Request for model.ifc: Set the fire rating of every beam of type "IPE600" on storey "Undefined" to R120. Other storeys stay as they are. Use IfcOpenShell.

First a look at what the model holds.

```python
import ifcopenshell
import ifcopenshell.util.element

model = ifcopenshell.open("model.ifc")
print(model.schema)
storey = next(s for s in model.by_type("IfcBuildingStorey") if s.Name == "Undefined")
beams = [e for e in ifcopenshell.util.element.get_decomposition(storey) if e.is_a("IfcBeam")]
seen = {}
for e in beams:
    element_type = ifcopenshell.util.element.get_type(e)
    key = (element_type.Name if element_type != e and element_type else None, ifcopenshell.util.element.get_pset(e, "Pset_BeamCommon", "FireRating"))
    seen[key] = seen.get(key, 0) + 1
for (name, value), count in sorted(seen.items(), key=str):
    print(count, "x", name, "|", value)
```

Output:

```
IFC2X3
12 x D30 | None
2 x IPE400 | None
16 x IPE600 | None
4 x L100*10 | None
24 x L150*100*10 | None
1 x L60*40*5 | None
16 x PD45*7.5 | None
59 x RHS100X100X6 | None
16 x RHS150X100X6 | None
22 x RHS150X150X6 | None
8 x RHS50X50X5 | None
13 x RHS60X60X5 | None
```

```python
import ifcopenshell
import ifcopenshell.api.pset
import ifcopenshell.util.element

model = ifcopenshell.open("model.ifc")

storey = next(s for s in model.by_type("IfcBuildingStorey") if s.Name == "Undefined")
beams = [e for e in ifcopenshell.util.element.get_decomposition(storey) if e.is_a("IfcBeam")]

count = 0
for e in beams:
    element_type = ifcopenshell.util.element.get_type(e)
    if element_type in (None, e) or element_type.Name != "IPE600":
        continue
    found = ifcopenshell.util.element.get_pset(e, "Pset_BeamCommon", should_inherit=False)
    if found:
        pset = model.by_id(found["id"])
        if len(ifcopenshell.util.element.get_elements_by_pset(pset)) > 1:
            pset = ifcopenshell.api.pset.unshare_pset(model, products=[e], pset=pset)[0]
    else:
        pset = ifcopenshell.api.pset.add_pset(model, product=e, name="Pset_BeamCommon")
    ifcopenshell.api.pset.edit_pset(model, pset=pset, properties={"FireRating": "R120"})
    count += 1

print(count, "beams updated")

model.write("model_updated.ifc")
```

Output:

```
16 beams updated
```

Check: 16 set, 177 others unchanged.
